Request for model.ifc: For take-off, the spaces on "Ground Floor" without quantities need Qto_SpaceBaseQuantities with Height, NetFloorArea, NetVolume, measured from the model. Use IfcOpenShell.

First a look at what the model holds.

```python
import ifcopenshell
import ifcopenshell.util.element
import ifcopenshell.util.unit

model = ifcopenshell.open("model.ifc")
print(model.schema)
for unit_type in ("LENGTHUNIT", "AREAUNIT", "VOLUMEUNIT"):
    print(unit_type, ifcopenshell.util.unit.calculate_unit_scale(model, unit_type))
storey = next(s for s in model.by_type("IfcBuildingStorey") if s.Name == "Ground Floor")
spaces = [e for e in ifcopenshell.util.element.get_decomposition(storey) if e.is_a("IfcSpace")]
for e in sorted(spaces, key=lambda e: e.id()):
    print(e.id(), e.is_a(), e.Name, list(ifcopenshell.util.element.get_psets(e, qtos_only=True)), sep=" | ")
```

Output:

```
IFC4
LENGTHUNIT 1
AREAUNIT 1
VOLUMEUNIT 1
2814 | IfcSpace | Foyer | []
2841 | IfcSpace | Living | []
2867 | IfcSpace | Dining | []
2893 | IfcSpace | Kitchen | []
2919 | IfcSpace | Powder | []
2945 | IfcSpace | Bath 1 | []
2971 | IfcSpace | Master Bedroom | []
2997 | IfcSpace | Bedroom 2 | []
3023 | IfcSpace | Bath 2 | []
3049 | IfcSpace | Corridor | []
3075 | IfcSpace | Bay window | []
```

```python
import ifcopenshell
import ifcopenshell.api.pset
import ifcopenshell.geom
import ifcopenshell.util.element
import ifcopenshell.util.shape
import ifcopenshell.util.unit

model = ifcopenshell.open("model.ifc")
unit_scale = ifcopenshell.util.unit.calculate_unit_scale(model)
area_scale = ifcopenshell.util.unit.calculate_unit_scale(model, "AREAUNIT")
volume_scale = ifcopenshell.util.unit.calculate_unit_scale(model, "VOLUMEUNIT")
settings = ifcopenshell.geom.settings()

storey = next(s for s in model.by_type("IfcBuildingStorey") if s.Name == "Ground Floor")
spaces = [e for e in ifcopenshell.util.element.get_decomposition(storey) if e.is_a("IfcSpace")]

for e in sorted(spaces, key=lambda e: e.id()):
    if ifcopenshell.util.element.get_psets(e, qtos_only=True, should_inherit=False):
        continue
    # Geometry comes back in metres, in the element's own axes.
    shape = ifcopenshell.geom.create_shape(settings, e)
    values = {
        "Height": ifcopenshell.util.shape.get_z(shape.geometry) / unit_scale,
        "NetFloorArea": ifcopenshell.util.shape.get_footprint_area(shape.geometry) / area_scale,
        "NetVolume": ifcopenshell.util.shape.get_volume(shape.geometry) / volume_scale,
    }
    qto = ifcopenshell.api.pset.add_qto(model, product=e, name="Qto_SpaceBaseQuantities")
    ifcopenshell.api.pset.edit_qto(model, qto=qto, properties=values)
    print(e.id(), {k: round(v, 3) for k, v in values.items()})

model.write("model_updated.ifc")
```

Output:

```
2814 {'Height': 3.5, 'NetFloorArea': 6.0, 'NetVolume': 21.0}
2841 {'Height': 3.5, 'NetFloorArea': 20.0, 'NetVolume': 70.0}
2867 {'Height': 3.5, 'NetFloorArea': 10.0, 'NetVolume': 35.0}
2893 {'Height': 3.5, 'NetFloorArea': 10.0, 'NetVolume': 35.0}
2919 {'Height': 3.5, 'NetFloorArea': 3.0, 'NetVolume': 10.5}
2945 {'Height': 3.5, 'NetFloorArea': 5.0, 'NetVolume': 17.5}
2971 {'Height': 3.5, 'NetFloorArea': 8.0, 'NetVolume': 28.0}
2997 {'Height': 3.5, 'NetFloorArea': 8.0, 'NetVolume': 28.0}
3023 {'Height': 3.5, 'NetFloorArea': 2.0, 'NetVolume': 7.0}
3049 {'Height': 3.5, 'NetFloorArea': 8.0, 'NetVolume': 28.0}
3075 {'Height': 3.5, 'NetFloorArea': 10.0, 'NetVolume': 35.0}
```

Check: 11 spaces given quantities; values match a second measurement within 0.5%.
